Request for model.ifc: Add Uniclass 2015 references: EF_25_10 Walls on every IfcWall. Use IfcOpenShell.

First a look at what the model holds.

```python
import ifcopenshell

model = ifcopenshell.open("model.ifc")
print(model.schema)
print("classifications:", [c.Name for c in model.by_type("IfcClassification")])
for ifc_class in ("IfcDoor", "IfcRoof", "IfcStair", "IfcWall", "IfcWindow"):
    print(ifc_class, len(model.by_type(ifc_class)))
```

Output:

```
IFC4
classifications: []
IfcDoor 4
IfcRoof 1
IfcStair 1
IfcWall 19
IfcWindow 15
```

```python
import ifcopenshell
import ifcopenshell.api.classification

model = ifcopenshell.open("model.ifc")

system = ifcopenshell.api.classification.add_classification(model, classification="Uniclass 2015")

codes = {
    "IfcWall": ("EF_25_10", "Walls"),
}
for ifc_class, (code, name) in codes.items():
    products = model.by_type(ifc_class)
    ifcopenshell.api.classification.add_reference(
        model, products=products, classification=system, identification=code, name=name
    )
    print(code, len(products))

model.write("model-out.ifc")
```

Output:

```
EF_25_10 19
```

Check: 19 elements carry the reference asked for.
